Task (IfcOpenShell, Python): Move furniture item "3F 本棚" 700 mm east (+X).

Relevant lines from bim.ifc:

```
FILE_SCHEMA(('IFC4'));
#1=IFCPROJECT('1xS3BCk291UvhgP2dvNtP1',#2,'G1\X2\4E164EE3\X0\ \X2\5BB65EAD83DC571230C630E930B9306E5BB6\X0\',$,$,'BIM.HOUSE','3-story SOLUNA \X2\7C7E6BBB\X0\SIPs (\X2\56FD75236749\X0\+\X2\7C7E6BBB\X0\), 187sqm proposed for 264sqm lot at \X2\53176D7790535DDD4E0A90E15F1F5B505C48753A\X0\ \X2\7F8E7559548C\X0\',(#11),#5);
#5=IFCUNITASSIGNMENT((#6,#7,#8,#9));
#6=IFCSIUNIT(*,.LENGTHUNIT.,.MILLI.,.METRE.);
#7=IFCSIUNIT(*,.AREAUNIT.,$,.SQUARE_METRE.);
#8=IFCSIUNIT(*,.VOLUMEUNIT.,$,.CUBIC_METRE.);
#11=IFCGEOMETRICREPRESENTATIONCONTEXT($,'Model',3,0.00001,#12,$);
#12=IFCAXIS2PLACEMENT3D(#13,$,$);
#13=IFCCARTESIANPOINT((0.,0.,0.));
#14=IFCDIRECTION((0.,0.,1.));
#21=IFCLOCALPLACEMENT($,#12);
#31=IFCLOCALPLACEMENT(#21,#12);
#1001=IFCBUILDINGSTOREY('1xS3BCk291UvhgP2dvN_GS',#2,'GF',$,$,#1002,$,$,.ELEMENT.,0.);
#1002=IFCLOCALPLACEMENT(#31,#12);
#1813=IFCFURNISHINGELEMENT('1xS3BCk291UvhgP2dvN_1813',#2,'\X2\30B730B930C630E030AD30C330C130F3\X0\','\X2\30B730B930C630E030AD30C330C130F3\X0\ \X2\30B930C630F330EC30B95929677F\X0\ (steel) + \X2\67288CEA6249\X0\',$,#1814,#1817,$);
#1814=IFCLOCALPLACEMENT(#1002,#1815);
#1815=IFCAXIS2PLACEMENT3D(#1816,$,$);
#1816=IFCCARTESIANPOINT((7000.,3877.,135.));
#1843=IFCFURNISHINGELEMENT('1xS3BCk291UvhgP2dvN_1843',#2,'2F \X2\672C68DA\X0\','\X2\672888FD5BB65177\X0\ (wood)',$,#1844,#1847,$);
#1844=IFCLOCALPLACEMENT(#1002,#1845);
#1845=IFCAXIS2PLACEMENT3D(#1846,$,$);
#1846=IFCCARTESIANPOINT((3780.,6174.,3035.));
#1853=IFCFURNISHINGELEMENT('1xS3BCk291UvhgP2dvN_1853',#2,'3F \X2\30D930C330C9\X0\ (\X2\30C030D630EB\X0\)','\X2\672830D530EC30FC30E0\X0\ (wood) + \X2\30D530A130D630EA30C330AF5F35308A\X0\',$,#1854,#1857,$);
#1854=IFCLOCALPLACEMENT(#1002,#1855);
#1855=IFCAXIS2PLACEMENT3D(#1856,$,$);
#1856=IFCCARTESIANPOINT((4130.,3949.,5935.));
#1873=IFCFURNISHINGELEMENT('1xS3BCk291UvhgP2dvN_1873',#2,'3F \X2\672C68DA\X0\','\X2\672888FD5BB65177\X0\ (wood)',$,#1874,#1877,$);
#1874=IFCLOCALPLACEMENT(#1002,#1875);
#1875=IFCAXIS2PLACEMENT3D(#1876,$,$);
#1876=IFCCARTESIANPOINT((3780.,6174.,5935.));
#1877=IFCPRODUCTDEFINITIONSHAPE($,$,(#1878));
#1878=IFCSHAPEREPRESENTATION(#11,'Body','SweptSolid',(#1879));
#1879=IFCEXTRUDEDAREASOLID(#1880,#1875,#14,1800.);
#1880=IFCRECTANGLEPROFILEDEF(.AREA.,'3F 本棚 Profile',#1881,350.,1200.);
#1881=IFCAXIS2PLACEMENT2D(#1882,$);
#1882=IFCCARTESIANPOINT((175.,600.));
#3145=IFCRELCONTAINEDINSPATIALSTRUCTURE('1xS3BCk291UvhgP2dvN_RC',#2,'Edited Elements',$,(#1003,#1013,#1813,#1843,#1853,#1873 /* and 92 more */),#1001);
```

```python
import ifcopenshell
import ifcopenshell.api.geometry
import ifcopenshell.util.placement
import ifcopenshell.util.unit

model = ifcopenshell.open("bim.ifc")
unit_scale = ifcopenshell.util.unit.calculate_unit_scale(model)

item = model.by_id(1873)
matrix = ifcopenshell.util.placement.get_local_placement(item.ObjectPlacement)
matrix[0, 3] += 0.7 / unit_scale
ifcopenshell.api.geometry.edit_object_placement(model, product=item, matrix=matrix, is_si=False)

print(ifcopenshell.util.placement.get_local_placement(item.ObjectPlacement).round(3) + 0.0)

model.write("bim-out.ifc")
```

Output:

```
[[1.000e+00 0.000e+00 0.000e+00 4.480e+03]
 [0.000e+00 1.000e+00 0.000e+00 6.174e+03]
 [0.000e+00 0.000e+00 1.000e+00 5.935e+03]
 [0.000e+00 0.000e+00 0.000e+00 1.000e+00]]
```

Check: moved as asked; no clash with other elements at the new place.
